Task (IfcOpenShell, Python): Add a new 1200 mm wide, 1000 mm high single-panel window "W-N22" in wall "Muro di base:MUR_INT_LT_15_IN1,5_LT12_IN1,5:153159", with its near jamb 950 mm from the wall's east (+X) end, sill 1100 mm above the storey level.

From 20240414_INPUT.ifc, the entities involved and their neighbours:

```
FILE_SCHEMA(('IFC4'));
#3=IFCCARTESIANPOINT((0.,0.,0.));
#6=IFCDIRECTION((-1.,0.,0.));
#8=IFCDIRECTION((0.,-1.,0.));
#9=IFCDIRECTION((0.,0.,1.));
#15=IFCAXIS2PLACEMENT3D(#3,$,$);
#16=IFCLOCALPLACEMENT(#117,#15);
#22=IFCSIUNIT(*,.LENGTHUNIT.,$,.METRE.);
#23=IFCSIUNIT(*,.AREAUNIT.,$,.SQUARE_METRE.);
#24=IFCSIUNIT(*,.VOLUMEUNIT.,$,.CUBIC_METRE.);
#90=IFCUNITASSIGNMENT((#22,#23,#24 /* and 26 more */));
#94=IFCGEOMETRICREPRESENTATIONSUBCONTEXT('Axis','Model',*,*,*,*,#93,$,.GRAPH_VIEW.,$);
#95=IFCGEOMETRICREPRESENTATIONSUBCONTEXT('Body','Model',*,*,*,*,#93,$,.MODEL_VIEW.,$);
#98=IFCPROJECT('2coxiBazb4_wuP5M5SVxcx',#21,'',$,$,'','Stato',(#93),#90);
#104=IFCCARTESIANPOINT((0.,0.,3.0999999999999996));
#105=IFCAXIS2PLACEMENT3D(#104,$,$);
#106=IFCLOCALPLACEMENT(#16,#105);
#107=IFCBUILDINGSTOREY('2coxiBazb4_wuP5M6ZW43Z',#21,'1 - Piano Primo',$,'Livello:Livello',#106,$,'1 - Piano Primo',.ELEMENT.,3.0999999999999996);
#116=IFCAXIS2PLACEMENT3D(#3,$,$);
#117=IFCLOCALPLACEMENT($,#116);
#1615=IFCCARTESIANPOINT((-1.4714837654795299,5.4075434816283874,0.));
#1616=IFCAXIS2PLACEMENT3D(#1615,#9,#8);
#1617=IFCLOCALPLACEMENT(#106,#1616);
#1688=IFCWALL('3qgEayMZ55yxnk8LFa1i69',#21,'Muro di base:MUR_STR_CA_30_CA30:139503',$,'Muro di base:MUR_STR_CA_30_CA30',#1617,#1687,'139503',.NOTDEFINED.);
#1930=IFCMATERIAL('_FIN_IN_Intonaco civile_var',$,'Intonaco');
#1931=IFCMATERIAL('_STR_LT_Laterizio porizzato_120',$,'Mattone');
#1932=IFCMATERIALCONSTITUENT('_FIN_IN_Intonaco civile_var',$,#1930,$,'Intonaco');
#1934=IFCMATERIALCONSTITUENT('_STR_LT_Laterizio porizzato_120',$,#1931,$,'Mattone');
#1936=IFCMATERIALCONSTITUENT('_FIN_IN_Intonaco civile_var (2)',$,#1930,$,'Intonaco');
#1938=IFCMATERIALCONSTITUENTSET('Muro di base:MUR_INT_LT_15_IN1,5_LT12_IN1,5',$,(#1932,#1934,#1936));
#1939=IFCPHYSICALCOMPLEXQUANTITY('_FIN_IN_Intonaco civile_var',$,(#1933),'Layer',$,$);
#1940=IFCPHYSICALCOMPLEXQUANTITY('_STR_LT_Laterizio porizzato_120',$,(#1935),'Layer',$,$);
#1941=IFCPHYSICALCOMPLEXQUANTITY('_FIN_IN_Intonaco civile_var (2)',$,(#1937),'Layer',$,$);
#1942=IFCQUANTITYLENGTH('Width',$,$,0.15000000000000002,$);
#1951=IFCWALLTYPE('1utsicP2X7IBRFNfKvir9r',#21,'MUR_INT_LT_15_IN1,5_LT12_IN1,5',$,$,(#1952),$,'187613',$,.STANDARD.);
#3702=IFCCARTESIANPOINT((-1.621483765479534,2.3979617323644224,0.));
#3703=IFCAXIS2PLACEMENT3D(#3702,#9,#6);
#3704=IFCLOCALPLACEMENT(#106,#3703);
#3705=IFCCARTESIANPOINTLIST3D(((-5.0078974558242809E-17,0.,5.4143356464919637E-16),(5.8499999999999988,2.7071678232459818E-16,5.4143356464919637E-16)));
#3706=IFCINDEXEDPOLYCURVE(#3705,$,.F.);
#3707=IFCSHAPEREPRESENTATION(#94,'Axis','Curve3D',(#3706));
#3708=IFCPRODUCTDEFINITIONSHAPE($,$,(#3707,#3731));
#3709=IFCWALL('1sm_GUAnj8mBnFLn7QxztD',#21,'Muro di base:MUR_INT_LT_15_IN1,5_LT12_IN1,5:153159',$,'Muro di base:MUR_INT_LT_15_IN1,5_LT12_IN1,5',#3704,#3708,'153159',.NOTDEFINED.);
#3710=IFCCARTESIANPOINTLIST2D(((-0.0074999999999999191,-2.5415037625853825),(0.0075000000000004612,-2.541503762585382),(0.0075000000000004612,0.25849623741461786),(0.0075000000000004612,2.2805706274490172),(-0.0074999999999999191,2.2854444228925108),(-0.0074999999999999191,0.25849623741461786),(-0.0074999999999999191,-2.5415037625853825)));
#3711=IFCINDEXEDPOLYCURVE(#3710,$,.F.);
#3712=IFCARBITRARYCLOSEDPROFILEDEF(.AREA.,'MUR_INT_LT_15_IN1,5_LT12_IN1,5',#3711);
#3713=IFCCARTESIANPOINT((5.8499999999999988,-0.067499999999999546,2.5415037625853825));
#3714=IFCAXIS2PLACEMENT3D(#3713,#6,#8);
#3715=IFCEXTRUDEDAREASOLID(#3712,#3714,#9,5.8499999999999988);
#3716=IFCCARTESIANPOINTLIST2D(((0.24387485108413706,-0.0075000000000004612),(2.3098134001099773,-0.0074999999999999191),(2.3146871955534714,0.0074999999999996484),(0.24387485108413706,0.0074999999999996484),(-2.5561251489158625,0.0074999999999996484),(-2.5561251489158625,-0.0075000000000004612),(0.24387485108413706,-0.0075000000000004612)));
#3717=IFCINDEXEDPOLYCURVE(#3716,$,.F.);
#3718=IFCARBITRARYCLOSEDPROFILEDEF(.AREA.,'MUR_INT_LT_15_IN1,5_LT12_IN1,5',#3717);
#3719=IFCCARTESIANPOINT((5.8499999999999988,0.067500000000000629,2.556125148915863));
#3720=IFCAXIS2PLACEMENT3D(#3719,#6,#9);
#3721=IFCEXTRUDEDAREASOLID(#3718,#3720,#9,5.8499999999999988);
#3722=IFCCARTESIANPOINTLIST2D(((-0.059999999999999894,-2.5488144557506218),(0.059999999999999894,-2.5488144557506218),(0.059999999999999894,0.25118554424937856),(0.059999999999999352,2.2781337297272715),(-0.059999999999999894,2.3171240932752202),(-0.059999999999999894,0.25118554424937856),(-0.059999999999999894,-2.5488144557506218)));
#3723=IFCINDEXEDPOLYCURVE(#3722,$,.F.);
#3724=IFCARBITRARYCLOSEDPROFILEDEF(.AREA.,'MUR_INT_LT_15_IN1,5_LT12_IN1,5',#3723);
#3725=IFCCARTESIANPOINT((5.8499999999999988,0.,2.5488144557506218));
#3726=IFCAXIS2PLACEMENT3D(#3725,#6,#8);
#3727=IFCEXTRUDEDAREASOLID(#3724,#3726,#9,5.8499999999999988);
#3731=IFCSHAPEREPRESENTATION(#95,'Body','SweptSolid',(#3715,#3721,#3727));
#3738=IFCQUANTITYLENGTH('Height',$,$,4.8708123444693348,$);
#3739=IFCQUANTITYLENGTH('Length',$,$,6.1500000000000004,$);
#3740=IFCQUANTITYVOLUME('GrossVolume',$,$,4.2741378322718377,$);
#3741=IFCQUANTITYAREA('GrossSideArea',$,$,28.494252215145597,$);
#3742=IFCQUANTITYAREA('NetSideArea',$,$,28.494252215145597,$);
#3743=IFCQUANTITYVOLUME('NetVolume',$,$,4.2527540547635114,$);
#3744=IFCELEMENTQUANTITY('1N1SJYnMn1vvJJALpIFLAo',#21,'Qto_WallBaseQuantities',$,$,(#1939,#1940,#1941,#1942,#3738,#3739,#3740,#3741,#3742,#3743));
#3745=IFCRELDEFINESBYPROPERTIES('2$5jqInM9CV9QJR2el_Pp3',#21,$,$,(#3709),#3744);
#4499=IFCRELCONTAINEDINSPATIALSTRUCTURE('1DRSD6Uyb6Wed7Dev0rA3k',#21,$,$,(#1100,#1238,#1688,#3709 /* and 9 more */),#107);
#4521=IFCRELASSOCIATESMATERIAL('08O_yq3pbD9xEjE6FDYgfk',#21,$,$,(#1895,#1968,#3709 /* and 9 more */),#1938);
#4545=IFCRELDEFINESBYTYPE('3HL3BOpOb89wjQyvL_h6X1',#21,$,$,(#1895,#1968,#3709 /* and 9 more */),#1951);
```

```python
import numpy as np
import ifcopenshell
import ifcopenshell.api.feature
import ifcopenshell.api.geometry
import ifcopenshell.api.pset
import ifcopenshell.api.root
import ifcopenshell.api.spatial
import ifcopenshell.geom
import ifcopenshell.util.element
import ifcopenshell.util.placement
import ifcopenshell.util.representation
import ifcopenshell.util.shape
import ifcopenshell.util.unit

model = ifcopenshell.open("20240414_INPUT.ifc")
unit_scale = ifcopenshell.util.unit.calculate_unit_scale(model)
area_scale = ifcopenshell.util.unit.calculate_unit_scale(model, "AREAUNIT")
volume_scale = ifcopenshell.util.unit.calculate_unit_scale(model, "VOLUMEUNIT")
settings = ifcopenshell.geom.settings()


def volume(element):
    """Net volume in cubic metres, openings subtracted."""
    shape = ifcopenshell.geom.create_shape(settings, element)
    return ifcopenshell.util.shape.get_volume(shape.geometry)


wall = model.by_guid("1sm_GUAnj8mBnFLn7QxztD")
storey = ifcopenshell.util.element.get_container(wall, ifc_class="IfcBuildingStorey")
context = ifcopenshell.util.representation.get_context(model, "Model", "Body", "MODEL_VIEW")
before = volume(wall)

width, height, from_end, sill = 1.2, 1, 0.95, 1.1  # metres

# The wall runs along its own X axis, and the end named is its -X end.
wall_shape = ifcopenshell.geom.create_shape(settings, wall)
x, y, z = ifcopenshell.util.shape.get_vertices(wall_shape.geometry).T
start = x.min() + from_end
face, thickness = float(y.min()), float(y.max() - y.min())
wall_matrix = ifcopenshell.util.placement.get_local_placement(wall.ObjectPlacement)
level = ifcopenshell.util.placement.get_local_placement(storey.ObjectPlacement)[2, 3]


def in_wall(x, y):
    """Placement at x, y metres in the wall's axes, at sill height."""
    matrix = wall_matrix.copy()
    matrix[:, 3] = wall_matrix @ np.array([x / unit_scale, y / unit_scale, 0.0, 1.0])
    matrix[2, 3] = level + sill / unit_scale
    return matrix


# Opening: a box that overshoots both wall faces by 50 mm.
opening = ifcopenshell.api.root.create_entity(model, ifc_class="IfcOpeningElement", predefined_type="OPENING")
box = ifcopenshell.api.geometry.add_wall_representation(
    model, context=context, length=width, height=height, thickness=thickness + 0.1
)
ifcopenshell.api.geometry.assign_representation(model, product=opening, representation=box)
ifcopenshell.api.geometry.edit_object_placement(model, product=opening, matrix=in_wall(start, face - 0.05), is_si=False)
ifcopenshell.api.feature.add_feature(model, feature=opening, element=wall)

window = ifcopenshell.api.root.create_entity(model, ifc_class="IfcWindow", name="W-N22", predefined_type="WINDOW")
window.OverallWidth, window.OverallHeight = width / unit_scale, height / unit_scale
window.PartitioningType = "SINGLE_PANEL"
body = ifcopenshell.api.geometry.add_window_representation(
    model,
    context=context,
    overall_width=window.OverallWidth,
    overall_height=window.OverallHeight,
    partition_type="SINGLE_PANEL",
)
ifcopenshell.api.geometry.assign_representation(model, product=window, representation=body)
ifcopenshell.api.spatial.assign_container(model, products=[window], relating_structure=storey)
ifcopenshell.api.feature.add_filling(model, opening=opening, element=window)

# Centre the window in the wall's thickness.
ifcopenshell.api.geometry.edit_object_placement(model, product=window, matrix=in_wall(start, face), is_si=False)
window_shape = ifcopenshell.geom.create_shape(settings, window)
depth = ifcopenshell.util.shape.get_vertices(window_shape.geometry)[:, 1]
offset = face + thickness / 2 - (depth.min() + depth.max()) / 2
ifcopenshell.api.geometry.edit_object_placement(model, product=window, matrix=in_wall(start, offset), is_si=False)

after = volume(wall)

# Update the wall's stored quantities.
qto = model.by_id(ifcopenshell.util.element.get_pset(wall, "Qto_WallBaseQuantities", should_inherit=False)["id"])
ifcopenshell.api.pset.edit_qto(model, qto=qto, properties={
    "NetSideArea": after / thickness / area_scale,
    "NetVolume": after / volume_scale,
})

print(f"wall volume {before:.3f} -> {after:.3f} m3")

model.write("20240414_INPUT-out.ifc")
```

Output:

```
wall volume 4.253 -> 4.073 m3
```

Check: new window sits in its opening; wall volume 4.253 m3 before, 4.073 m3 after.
